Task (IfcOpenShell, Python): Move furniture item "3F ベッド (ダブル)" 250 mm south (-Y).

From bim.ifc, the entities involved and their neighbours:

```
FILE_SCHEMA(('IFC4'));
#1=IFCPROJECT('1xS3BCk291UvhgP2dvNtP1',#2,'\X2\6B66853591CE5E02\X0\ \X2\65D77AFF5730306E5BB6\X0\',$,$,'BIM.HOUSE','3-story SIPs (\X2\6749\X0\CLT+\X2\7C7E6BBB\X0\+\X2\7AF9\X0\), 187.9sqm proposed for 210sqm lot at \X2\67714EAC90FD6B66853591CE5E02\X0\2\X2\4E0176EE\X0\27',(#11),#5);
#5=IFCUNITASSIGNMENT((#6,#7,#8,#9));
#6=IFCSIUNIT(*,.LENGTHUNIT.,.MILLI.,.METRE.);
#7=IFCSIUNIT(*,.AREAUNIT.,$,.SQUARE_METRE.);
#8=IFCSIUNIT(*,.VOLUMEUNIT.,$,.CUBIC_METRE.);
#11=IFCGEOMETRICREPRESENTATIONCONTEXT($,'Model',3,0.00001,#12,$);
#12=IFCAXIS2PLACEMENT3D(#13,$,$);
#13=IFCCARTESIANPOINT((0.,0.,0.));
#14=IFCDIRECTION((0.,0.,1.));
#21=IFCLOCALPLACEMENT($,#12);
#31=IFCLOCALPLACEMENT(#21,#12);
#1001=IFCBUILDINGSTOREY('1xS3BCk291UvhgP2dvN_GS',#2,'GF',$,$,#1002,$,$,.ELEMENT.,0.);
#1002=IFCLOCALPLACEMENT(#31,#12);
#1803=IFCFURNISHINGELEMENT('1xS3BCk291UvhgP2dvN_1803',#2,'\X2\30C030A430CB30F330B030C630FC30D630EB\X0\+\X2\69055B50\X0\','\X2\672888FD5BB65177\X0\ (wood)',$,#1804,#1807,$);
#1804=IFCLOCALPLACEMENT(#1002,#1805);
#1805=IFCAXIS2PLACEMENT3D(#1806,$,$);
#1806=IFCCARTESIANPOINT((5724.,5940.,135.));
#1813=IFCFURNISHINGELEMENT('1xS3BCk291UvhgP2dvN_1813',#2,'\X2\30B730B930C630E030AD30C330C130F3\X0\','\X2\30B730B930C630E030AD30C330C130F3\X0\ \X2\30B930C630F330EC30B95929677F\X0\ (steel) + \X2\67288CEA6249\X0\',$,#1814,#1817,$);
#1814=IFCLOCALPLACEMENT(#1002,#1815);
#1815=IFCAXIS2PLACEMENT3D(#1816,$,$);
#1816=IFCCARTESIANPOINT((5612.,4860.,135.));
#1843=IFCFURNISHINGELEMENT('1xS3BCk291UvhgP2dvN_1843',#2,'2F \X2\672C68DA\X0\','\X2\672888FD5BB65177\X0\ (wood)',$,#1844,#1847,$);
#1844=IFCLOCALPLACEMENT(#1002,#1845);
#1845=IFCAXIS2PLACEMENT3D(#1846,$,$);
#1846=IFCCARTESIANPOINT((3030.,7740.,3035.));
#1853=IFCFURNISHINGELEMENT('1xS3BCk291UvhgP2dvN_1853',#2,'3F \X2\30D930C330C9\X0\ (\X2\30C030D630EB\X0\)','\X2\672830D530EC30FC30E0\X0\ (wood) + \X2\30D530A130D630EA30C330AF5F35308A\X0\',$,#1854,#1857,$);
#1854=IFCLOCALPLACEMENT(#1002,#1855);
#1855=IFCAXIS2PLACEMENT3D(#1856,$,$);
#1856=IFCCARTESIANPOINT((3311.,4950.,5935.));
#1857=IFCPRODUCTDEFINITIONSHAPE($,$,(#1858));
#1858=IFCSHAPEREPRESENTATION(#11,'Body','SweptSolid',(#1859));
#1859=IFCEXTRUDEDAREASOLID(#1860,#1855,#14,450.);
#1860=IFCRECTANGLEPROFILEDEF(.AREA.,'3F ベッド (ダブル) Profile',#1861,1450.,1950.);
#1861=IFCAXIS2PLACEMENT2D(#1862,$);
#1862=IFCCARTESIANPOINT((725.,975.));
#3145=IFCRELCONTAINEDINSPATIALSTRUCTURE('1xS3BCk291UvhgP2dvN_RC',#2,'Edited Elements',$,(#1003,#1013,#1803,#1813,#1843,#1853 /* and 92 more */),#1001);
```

```python
import ifcopenshell
import ifcopenshell.api.geometry
import ifcopenshell.util.placement
import ifcopenshell.util.unit

model = ifcopenshell.open("bim.ifc")
unit_scale = ifcopenshell.util.unit.calculate_unit_scale(model)

item = model.by_guid("1xS3BCk291UvhgP2dvN_1853")
matrix = ifcopenshell.util.placement.get_local_placement(item.ObjectPlacement)
matrix[1, 3] -= 0.25 / unit_scale
ifcopenshell.api.geometry.edit_object_placement(model, product=item, matrix=matrix, is_si=False)

print(ifcopenshell.util.placement.get_local_placement(item.ObjectPlacement).round(3) + 0.0)

model.write("bim_updated.ifc")
```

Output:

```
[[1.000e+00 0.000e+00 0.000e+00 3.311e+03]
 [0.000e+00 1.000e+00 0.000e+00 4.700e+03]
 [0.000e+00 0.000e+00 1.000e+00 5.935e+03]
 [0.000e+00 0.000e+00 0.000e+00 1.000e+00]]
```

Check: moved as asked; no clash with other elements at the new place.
